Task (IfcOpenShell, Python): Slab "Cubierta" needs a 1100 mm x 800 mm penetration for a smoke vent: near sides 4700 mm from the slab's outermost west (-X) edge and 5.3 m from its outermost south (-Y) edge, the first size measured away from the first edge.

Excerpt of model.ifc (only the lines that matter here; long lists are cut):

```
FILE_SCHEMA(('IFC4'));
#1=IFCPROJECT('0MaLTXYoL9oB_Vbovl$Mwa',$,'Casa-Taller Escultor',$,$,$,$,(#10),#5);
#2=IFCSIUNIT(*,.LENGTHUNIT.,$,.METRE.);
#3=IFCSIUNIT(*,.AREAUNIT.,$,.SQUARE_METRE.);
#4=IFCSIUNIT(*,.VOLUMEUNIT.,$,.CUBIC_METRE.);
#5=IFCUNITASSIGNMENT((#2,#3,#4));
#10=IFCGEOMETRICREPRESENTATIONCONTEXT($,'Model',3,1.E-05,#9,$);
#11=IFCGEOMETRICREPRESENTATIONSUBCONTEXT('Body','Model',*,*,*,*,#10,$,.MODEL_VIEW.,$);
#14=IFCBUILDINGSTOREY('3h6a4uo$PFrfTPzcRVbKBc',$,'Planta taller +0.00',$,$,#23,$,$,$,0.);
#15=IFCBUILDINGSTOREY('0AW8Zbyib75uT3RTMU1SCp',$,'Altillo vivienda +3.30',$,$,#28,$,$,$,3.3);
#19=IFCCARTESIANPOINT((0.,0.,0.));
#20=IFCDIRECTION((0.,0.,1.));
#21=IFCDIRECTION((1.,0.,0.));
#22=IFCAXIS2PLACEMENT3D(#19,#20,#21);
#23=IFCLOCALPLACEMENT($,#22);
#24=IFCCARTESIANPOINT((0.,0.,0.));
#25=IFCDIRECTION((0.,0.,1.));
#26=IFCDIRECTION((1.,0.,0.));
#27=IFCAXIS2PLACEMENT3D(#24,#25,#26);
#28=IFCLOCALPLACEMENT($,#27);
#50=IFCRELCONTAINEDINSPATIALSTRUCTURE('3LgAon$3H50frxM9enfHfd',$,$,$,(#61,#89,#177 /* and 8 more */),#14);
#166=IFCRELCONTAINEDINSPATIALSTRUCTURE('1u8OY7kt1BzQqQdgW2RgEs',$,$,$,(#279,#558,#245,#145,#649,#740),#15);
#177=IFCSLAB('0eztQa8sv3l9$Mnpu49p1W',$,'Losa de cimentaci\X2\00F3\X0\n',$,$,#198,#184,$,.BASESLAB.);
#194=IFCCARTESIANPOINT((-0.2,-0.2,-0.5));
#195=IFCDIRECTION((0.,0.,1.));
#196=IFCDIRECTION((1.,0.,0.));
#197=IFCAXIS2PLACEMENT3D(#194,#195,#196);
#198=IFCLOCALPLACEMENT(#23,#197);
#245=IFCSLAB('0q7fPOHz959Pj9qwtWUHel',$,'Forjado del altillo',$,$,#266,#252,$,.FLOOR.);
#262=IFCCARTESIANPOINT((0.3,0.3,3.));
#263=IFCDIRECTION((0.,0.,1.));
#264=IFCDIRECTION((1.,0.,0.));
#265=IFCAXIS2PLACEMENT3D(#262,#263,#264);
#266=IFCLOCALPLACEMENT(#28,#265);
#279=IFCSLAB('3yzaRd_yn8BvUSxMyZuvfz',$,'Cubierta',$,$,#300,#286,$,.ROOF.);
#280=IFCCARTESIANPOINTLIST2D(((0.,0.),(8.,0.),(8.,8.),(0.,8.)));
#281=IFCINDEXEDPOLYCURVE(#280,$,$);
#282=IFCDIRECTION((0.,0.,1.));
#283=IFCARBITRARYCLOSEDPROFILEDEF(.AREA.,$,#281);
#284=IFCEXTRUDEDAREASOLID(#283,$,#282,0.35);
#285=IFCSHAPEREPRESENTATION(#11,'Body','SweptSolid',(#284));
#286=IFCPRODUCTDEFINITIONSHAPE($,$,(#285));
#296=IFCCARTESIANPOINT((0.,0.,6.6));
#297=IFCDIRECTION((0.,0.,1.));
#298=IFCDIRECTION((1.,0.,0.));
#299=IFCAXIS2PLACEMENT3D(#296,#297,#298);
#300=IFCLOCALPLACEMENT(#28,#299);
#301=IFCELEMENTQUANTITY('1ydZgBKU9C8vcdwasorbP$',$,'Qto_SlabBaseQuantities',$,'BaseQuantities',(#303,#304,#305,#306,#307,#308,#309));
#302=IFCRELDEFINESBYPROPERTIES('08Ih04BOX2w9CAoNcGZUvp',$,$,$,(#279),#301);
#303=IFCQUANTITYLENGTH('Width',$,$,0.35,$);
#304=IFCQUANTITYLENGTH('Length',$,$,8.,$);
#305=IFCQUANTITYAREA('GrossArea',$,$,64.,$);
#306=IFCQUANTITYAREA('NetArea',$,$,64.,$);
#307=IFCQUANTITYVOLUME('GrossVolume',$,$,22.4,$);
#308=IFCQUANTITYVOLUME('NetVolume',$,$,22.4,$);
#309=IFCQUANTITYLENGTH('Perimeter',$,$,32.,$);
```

```python
import numpy as np
import ifcopenshell
import ifcopenshell.api.feature
import ifcopenshell.api.geometry
import ifcopenshell.api.pset
import ifcopenshell.api.root
import ifcopenshell.geom
import ifcopenshell.util.element
import ifcopenshell.util.placement
import ifcopenshell.util.representation
import ifcopenshell.util.shape
import ifcopenshell.util.unit

model = ifcopenshell.open("model.ifc")
unit_scale = ifcopenshell.util.unit.calculate_unit_scale(model)
area_scale = ifcopenshell.util.unit.calculate_unit_scale(model, "AREAUNIT")
volume_scale = ifcopenshell.util.unit.calculate_unit_scale(model, "VOLUMEUNIT")
settings = ifcopenshell.geom.settings()


def volume(element):
    """Net volume in cubic metres, openings subtracted."""
    shape = ifcopenshell.geom.create_shape(settings, element)
    return ifcopenshell.util.shape.get_volume(shape.geometry)


slab = model.by_guid("3yzaRd_yn8BvUSxMyZuvfz")
before = volume(slab)

# Extent in the slab's own axes, in metres. The edges named are its -X and -Y sides.
slab_shape = ifcopenshell.geom.create_shape(settings, slab)
vertices = ifcopenshell.util.shape.get_vertices(slab_shape.geometry)
x_min, y_min, bottom = vertices.min(axis=0)
top = vertices[:, 2].max()

opening = ifcopenshell.api.root.create_entity(model, ifc_class="IfcOpeningElement", name="Smoke vent opening", predefined_type="OPENING")
context = ifcopenshell.util.representation.get_context(model, "Model", "Body", "MODEL_VIEW")
width, depth = 1.1, 0.8
outline = [(0.0, 0.0), (width, 0.0), (width, depth), (0.0, depth), (0.0, 0.0)]
# Overshoot both faces by 50 mm so the cut is clean.
shape = ifcopenshell.api.geometry.add_slab_representation(
    model, context=context, depth=top - bottom + 0.1, polyline=outline
)
ifcopenshell.api.geometry.assign_representation(model, product=opening, representation=shape)

matrix = ifcopenshell.util.placement.get_local_placement(slab.ObjectPlacement)
matrix[:, 3] = matrix @ np.append(np.array([x_min + 4.7, y_min + 5.3, bottom - 0.05]) / unit_scale, 1.0)
ifcopenshell.api.geometry.edit_object_placement(model, product=opening, matrix=matrix, is_si=False)
ifcopenshell.api.feature.add_feature(model, feature=opening, element=slab)

after = volume(slab)

# Update the slab's stored quantities.
qto = model.by_id(ifcopenshell.util.element.get_pset(slab, "Qto_SlabBaseQuantities", should_inherit=False)["id"])
ifcopenshell.api.pset.edit_qto(model, qto=qto, properties={
    "NetArea": after / (top - bottom) / area_scale,
    "NetVolume": after / volume_scale,
})

print(f"slab volume {before:.3f} -> {after:.3f} m3")

model.write("model-out.ifc")
```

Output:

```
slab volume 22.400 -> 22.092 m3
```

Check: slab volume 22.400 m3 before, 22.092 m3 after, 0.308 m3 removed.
